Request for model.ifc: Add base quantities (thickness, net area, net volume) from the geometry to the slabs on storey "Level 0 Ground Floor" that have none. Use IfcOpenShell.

First a look at what the model holds.

```python
import ifcopenshell
import ifcopenshell.util.element
import ifcopenshell.util.unit

model = ifcopenshell.open("model.ifc")
print(model.schema)
for unit_type in ("LENGTHUNIT", "AREAUNIT", "VOLUMEUNIT"):
    print(unit_type, ifcopenshell.util.unit.calculate_unit_scale(model, unit_type))
storey = next(s for s in model.by_type("IfcBuildingStorey") if s.Name == "Level 0 Ground Floor")
slabs = [e for e in ifcopenshell.util.element.get_decomposition(storey) if e.is_a("IfcSlab")]
for e in sorted(slabs, key=lambda e: e.id()):
    print(e.id(), e.is_a(), e.Name, list(ifcopenshell.util.element.get_psets(e, qtos_only=True)), sep=" | ")
```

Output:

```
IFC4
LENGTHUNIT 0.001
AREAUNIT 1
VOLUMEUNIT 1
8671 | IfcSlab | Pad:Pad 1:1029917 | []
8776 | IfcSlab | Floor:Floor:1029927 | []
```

```python
import ifcopenshell
import ifcopenshell.api.pset
import ifcopenshell.geom
import ifcopenshell.util.element
import ifcopenshell.util.shape
import ifcopenshell.util.unit

model = ifcopenshell.open("model.ifc")
unit_scale = ifcopenshell.util.unit.calculate_unit_scale(model)
area_scale = ifcopenshell.util.unit.calculate_unit_scale(model, "AREAUNIT")
volume_scale = ifcopenshell.util.unit.calculate_unit_scale(model, "VOLUMEUNIT")
settings = ifcopenshell.geom.settings()

storey = next(s for s in model.by_type("IfcBuildingStorey") if s.Name == "Level 0 Ground Floor")
slabs = [e for e in ifcopenshell.util.element.get_decomposition(storey) if e.is_a("IfcSlab")]

for e in sorted(slabs, key=lambda e: e.id()):
    if ifcopenshell.util.element.get_psets(e, qtos_only=True, should_inherit=False):
        continue
    # Geometry comes back in metres, in the element's own axes.
    shape = ifcopenshell.geom.create_shape(settings, e)
    values = {
        "Width": ifcopenshell.util.shape.get_z(shape.geometry) / unit_scale,
        "NetArea": ifcopenshell.util.shape.get_footprint_area(shape.geometry) / area_scale,
        "NetVolume": ifcopenshell.util.shape.get_volume(shape.geometry) / volume_scale,
    }
    qto = ifcopenshell.api.pset.add_qto(model, product=e, name="Qto_SlabBaseQuantities")
    ifcopenshell.api.pset.edit_qto(model, qto=qto, properties=values)
    print(e.id(), {k: round(v, 3) for k, v in values.items()})

model.write("model_updated.ifc")
```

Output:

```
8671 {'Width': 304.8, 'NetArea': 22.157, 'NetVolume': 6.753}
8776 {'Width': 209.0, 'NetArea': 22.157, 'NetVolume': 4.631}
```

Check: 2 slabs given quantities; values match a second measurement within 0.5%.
